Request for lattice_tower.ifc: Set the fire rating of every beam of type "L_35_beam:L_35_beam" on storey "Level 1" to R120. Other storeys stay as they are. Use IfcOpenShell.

First a look at what the model holds.

```python
import ifcopenshell
import ifcopenshell.util.element

model = ifcopenshell.open("lattice_tower.ifc")
print(model.schema)
storey = next(s for s in model.by_type("IfcBuildingStorey") if s.Name == "Level 1")
beams = [e for e in ifcopenshell.util.element.get_decomposition(storey) if e.is_a("IfcBeam")]
seen = {}
for e in beams:
    element_type = ifcopenshell.util.element.get_type(e)
    key = (element_type.Name if element_type != e and element_type else None, ifcopenshell.util.element.get_pset(e, "Pset_BeamCommon", "FireRating"))
    seen[key] = seen.get(key, 0) + 1
for (name, value), count in sorted(seen.items(), key=str):
    print(count, "x", name, "|", value)
```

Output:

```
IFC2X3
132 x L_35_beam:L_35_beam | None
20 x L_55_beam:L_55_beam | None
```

```python
import ifcopenshell
import ifcopenshell.api.pset
import ifcopenshell.util.element

model = ifcopenshell.open("lattice_tower.ifc")

storey = next(s for s in model.by_type("IfcBuildingStorey") if s.Name == "Level 1")
beams = [e for e in ifcopenshell.util.element.get_decomposition(storey) if e.is_a("IfcBeam")]

count = 0
for e in beams:
    element_type = ifcopenshell.util.element.get_type(e)
    if element_type in (None, e) or element_type.Name != "L_35_beam:L_35_beam":
        continue
    # add_pset returns the element's existing set when there is one.
    pset = ifcopenshell.api.pset.add_pset(model, product=e, name="Pset_BeamCommon")
    ifcopenshell.api.pset.edit_pset(model, pset=pset, properties={"FireRating": "R120"})
    count += 1

print(count, "beams updated")

model.write("lattice_tower-out.ifc")
```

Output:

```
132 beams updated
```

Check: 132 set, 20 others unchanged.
